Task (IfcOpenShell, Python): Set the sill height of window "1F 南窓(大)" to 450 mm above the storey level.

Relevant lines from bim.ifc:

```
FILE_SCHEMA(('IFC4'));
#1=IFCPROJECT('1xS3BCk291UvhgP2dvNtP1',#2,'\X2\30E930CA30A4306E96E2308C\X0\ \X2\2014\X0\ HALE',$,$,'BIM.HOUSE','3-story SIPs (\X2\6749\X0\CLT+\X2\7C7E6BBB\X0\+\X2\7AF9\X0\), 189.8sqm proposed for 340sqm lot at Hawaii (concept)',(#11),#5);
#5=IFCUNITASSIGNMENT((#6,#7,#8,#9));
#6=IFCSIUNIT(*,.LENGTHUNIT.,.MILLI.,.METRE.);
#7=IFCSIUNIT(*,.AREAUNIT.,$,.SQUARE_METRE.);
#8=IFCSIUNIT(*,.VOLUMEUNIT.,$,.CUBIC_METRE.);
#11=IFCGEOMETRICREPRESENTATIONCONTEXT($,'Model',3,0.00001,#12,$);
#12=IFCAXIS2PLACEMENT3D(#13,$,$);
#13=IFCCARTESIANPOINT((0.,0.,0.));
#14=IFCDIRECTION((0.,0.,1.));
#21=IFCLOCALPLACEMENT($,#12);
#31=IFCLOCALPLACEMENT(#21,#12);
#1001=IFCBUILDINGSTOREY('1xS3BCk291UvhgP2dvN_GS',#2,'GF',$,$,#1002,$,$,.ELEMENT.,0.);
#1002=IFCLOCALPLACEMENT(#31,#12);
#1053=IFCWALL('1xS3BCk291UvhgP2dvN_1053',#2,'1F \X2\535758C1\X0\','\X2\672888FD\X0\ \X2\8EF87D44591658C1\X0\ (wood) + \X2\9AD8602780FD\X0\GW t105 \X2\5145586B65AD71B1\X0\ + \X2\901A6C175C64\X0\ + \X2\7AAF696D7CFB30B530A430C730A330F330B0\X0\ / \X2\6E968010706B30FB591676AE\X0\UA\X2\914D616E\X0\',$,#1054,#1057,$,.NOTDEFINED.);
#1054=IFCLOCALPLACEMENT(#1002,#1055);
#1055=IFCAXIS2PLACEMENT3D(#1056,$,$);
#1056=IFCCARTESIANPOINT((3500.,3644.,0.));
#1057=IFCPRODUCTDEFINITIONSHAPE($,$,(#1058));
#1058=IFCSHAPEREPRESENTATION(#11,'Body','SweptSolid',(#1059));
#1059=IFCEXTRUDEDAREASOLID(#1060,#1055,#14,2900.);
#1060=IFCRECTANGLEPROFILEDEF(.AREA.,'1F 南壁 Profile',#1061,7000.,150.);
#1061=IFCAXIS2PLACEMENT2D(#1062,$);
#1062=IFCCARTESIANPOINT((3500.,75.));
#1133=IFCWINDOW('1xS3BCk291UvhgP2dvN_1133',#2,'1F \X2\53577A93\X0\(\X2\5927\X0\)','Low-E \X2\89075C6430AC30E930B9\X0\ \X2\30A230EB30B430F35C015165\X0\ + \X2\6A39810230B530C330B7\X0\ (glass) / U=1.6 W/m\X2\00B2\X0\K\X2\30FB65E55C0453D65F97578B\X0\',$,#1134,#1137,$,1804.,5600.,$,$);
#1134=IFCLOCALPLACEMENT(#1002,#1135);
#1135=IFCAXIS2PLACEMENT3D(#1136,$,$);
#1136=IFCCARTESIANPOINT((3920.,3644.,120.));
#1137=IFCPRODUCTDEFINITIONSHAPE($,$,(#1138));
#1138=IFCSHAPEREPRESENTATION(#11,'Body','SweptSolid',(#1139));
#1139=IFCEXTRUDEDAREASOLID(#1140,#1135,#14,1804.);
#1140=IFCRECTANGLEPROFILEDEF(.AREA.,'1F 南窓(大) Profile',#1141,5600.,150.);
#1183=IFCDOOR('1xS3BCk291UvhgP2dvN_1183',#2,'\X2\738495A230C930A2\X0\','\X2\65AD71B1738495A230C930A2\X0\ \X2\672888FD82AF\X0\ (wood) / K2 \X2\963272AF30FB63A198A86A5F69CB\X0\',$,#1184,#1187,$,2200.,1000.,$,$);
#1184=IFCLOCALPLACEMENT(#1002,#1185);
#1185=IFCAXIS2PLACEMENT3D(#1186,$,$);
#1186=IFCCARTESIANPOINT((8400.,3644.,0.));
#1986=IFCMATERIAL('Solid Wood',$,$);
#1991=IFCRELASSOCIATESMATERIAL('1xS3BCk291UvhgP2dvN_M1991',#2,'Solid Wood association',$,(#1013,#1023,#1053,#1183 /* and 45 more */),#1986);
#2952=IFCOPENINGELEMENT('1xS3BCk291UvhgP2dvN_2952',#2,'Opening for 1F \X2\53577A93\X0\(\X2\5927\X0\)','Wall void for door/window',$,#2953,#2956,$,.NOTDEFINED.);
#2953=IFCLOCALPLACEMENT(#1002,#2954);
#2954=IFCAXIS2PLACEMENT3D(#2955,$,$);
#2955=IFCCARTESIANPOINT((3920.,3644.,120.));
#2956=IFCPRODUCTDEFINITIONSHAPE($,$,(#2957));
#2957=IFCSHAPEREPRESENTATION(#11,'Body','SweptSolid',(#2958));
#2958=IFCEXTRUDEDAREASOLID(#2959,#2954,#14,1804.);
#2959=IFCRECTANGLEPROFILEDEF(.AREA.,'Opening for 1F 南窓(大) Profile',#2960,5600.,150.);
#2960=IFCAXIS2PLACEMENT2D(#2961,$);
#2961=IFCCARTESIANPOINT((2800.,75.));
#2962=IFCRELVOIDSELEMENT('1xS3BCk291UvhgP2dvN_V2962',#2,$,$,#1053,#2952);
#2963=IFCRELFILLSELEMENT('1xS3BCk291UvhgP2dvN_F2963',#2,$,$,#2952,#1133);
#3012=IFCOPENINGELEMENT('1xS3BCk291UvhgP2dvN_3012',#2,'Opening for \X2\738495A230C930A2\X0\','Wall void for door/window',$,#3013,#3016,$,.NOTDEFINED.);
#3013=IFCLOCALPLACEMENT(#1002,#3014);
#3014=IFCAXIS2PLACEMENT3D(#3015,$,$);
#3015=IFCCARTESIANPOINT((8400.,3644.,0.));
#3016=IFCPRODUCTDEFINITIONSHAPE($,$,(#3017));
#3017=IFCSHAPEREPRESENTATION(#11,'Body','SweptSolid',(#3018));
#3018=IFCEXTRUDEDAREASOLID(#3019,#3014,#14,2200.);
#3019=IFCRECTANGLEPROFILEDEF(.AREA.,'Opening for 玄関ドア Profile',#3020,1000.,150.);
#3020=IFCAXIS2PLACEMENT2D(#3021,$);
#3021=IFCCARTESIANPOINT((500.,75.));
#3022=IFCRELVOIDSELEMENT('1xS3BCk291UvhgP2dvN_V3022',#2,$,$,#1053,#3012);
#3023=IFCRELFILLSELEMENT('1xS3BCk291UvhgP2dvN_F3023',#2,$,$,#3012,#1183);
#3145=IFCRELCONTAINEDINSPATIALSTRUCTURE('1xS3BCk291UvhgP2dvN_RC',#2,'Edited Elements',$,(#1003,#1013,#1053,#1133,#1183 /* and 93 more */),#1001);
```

```python
import numpy as np
import ifcopenshell
import ifcopenshell.api.geometry
import ifcopenshell.geom
import ifcopenshell.util.element
import ifcopenshell.util.placement
import ifcopenshell.util.shape
import ifcopenshell.util.unit

model = ifcopenshell.open("bim.ifc")
unit_scale = ifcopenshell.util.unit.calculate_unit_scale(model)

window = model.by_guid("1xS3BCk291UvhgP2dvN_1133")
opening = window.FillsVoids[0].RelatingOpeningElement
storey = ifcopenshell.util.element.get_container(window, ifc_class="IfcBuildingStorey")
level = ifcopenshell.util.placement.get_local_placement(storey.ObjectPlacement)[2, 3]

# The opening's origin need not be at the sill, so measure its lowest point.
shape = ifcopenshell.geom.create_shape(ifcopenshell.geom.settings(), opening)
bottom = ifcopenshell.util.shape.get_shape_bottom_elevation(shape, shape.geometry) / unit_scale
dz = level + 450.0 - bottom

shift = np.array([0.0, 0.0, dz])
# The window is not placed relative to its opening, so move both.
for product in (opening, window):
    matrix = ifcopenshell.util.placement.get_local_placement(product.ObjectPlacement)
    matrix[:3, 3] += shift
    ifcopenshell.api.geometry.edit_object_placement(model, product=product, matrix=matrix, is_si=False)

print(f"moved by {dz * unit_scale:+.3f} m")

model.write("bim_v2.ifc")
```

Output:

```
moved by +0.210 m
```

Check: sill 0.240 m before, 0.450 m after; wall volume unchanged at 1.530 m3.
